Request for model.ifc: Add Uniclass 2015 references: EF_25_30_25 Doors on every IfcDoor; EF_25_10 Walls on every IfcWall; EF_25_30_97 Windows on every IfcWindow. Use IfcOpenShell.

First a look at what the model holds.

```python
import ifcopenshell

model = ifcopenshell.open("model.ifc")
print(model.schema)
print("classifications:", [c.Name for c in model.by_type("IfcClassification")])
for ifc_class in ("IfcDoor", "IfcRoof", "IfcStair", "IfcWall", "IfcWindow"):
    print(ifc_class, len(model.by_type(ifc_class)))
```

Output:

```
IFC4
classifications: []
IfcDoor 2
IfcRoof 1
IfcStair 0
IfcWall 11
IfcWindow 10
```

```python
import ifcopenshell
import ifcopenshell.api.classification

model = ifcopenshell.open("model.ifc")

system = ifcopenshell.api.classification.add_classification(model, classification="Uniclass 2015")

codes = {
    "IfcDoor": ("EF_25_30_25", "Doors"),
    "IfcWall": ("EF_25_10", "Walls"),
    "IfcWindow": ("EF_25_30_97", "Windows"),
}
for ifc_class, (code, name) in codes.items():
    products = model.by_type(ifc_class)
    ifcopenshell.api.classification.add_reference(
        model, products=products, classification=system, identification=code, name=name
    )
    print(code, len(products))

model.write("model_v2.ifc")
```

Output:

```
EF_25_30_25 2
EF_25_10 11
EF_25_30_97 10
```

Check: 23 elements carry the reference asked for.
